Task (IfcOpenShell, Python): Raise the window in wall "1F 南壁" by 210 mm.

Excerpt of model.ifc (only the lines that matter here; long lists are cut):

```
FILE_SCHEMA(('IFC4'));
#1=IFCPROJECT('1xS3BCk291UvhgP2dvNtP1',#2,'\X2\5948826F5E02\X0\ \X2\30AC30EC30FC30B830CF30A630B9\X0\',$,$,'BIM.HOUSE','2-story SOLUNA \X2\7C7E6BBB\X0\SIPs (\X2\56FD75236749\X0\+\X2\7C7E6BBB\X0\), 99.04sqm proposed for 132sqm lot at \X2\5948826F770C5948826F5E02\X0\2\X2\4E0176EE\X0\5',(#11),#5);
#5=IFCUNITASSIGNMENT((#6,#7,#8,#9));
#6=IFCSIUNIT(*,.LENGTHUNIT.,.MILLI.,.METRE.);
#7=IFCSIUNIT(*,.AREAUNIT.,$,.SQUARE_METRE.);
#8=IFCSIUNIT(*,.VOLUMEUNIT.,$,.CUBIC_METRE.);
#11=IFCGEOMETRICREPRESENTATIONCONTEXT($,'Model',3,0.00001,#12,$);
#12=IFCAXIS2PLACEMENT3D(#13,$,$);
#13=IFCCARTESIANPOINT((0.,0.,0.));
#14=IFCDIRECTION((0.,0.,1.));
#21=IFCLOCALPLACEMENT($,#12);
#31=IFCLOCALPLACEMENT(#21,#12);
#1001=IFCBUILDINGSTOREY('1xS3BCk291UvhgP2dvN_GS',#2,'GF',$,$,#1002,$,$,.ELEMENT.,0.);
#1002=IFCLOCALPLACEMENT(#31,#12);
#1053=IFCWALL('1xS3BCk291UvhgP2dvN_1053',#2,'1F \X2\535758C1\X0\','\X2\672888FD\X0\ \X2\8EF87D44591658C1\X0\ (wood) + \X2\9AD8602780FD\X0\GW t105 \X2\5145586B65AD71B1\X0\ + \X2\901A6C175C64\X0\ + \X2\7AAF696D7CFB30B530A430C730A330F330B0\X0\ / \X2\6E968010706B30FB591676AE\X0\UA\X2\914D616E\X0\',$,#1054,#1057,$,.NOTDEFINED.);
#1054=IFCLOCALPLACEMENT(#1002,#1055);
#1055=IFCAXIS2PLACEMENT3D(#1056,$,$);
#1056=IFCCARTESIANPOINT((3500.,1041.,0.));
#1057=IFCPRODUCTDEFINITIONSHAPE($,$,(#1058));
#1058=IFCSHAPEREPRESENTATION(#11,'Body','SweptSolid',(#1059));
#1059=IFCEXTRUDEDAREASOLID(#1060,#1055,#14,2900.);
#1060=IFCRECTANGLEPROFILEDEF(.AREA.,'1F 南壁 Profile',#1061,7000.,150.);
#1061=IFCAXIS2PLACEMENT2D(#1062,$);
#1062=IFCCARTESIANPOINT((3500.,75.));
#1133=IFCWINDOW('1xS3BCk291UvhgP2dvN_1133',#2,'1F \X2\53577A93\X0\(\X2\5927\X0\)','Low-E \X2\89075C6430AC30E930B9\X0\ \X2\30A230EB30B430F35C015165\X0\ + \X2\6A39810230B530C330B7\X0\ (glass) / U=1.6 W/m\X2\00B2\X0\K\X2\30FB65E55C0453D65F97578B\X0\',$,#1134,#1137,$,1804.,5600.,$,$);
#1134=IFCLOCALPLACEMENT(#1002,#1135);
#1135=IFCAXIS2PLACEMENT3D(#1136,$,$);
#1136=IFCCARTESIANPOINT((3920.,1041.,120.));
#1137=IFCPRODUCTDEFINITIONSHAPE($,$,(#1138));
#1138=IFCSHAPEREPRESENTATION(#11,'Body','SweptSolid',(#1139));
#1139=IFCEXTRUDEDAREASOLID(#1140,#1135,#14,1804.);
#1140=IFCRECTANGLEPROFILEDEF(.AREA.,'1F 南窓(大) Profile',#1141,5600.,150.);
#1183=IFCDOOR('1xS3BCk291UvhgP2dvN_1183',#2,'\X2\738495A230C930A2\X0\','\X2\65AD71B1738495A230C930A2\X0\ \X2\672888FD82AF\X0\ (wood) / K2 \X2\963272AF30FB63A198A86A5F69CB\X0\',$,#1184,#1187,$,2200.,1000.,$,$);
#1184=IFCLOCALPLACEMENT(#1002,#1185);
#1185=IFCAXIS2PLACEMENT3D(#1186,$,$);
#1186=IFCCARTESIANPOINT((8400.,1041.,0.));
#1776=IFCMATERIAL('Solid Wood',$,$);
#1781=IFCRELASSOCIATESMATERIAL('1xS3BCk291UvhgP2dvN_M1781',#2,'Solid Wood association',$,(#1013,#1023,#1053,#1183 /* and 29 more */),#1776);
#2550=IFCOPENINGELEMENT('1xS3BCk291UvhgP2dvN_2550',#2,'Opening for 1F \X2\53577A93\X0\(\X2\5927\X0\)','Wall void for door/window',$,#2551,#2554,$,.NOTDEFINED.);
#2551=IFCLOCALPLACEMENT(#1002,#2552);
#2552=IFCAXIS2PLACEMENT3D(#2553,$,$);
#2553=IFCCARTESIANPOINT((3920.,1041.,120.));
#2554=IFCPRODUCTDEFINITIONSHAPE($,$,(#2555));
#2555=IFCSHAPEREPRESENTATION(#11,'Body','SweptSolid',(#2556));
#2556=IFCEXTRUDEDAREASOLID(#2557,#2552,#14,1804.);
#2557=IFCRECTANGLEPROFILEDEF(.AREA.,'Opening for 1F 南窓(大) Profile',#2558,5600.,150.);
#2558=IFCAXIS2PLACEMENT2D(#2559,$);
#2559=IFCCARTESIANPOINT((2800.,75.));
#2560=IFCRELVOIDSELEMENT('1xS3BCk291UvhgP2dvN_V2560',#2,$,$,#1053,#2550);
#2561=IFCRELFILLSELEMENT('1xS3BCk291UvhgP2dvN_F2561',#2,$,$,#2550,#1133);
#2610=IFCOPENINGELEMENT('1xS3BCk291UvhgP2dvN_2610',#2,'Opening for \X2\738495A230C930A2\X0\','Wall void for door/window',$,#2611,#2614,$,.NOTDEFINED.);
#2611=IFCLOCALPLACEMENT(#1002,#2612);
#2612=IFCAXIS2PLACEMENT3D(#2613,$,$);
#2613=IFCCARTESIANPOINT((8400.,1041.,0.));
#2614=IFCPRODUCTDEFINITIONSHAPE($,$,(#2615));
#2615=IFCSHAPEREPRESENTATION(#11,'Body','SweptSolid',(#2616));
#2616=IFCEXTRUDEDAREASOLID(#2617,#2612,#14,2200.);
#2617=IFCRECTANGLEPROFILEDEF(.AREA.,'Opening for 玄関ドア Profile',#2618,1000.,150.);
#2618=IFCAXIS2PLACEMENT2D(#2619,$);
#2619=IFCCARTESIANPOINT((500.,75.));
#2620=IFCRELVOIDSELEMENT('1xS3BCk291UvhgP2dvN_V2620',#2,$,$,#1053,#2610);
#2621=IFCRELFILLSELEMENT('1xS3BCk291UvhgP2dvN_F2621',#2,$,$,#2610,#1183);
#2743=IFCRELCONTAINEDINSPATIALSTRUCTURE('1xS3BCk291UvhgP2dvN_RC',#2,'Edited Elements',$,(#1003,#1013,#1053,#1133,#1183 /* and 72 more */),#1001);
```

```python
import numpy as np
import ifcopenshell
import ifcopenshell.api.geometry
import ifcopenshell.util.placement
import ifcopenshell.util.unit

model = ifcopenshell.open("model.ifc")
unit_scale = ifcopenshell.util.unit.calculate_unit_scale(model)

window = model.by_guid("1xS3BCk291UvhgP2dvN_1133")
opening = window.FillsVoids[0].RelatingOpeningElement
dz = 0.21 / unit_scale

shift = np.array([0.0, 0.0, dz])
# The window is not placed relative to its opening, so move both.
for product in (opening, window):
    matrix = ifcopenshell.util.placement.get_local_placement(product.ObjectPlacement)
    matrix[:3, 3] += shift
    ifcopenshell.api.geometry.edit_object_placement(model, product=product, matrix=matrix, is_si=False)

print(f"moved by {dz * unit_scale:+.3f} m")

model.write("model_rev.ifc")
```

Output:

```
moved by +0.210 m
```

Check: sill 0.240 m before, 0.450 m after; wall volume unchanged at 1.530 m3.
